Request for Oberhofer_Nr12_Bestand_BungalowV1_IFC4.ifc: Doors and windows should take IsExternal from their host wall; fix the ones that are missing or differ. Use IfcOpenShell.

First a look at what the model holds.

```python
import ifcopenshell
import ifcopenshell.util.element

model = ifcopenshell.open("Oberhofer_Nr12_Bestand_BungalowV1_IFC4.ifc")
print(model.schema)
seen = {}
for e in model.by_type("IfcDoor") + model.by_type("IfcWindow"):
    if not e.FillsVoids:
        continue
    host = e.FillsVoids[0].RelatingOpeningElement.VoidsElements[0].RelatingBuildingElement
    own = ifcopenshell.util.element.get_pset(e, f"Pset_{e.is_a()[3:].removesuffix('StandardCase')}Common", "IsExternal")
    wall = ifcopenshell.util.element.get_pset(host, "Pset_WallCommon", "IsExternal")
    seen[e.is_a(), own, wall] = seen.get((e.is_a(), own, wall), 0) + 1
for (cls, own, wall), count in sorted(seen.items(), key=str):
    print(count, cls, "IsExternal:", own, "| host wall:", wall)
```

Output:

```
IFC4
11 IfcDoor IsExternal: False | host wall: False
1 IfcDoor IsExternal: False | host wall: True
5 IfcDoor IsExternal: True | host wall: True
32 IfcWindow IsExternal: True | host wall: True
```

```python
import ifcopenshell
import ifcopenshell.api.pset
import ifcopenshell.util.element

model = ifcopenshell.open("Oberhofer_Nr12_Bestand_BungalowV1_IFC4.ifc")

count = 0
for ifc_class, pset_name in (("IfcDoor", "Pset_DoorCommon"), ("IfcWindow", "Pset_WindowCommon")):
    for e in model.by_type(ifc_class):
        if not e.FillsVoids:
            continue
        host = e.FillsVoids[0].RelatingOpeningElement.VoidsElements[0].RelatingBuildingElement
        external = ifcopenshell.util.element.get_pset(host, "Pset_WallCommon", "IsExternal")
        if external is None or ifcopenshell.util.element.get_pset(e, pset_name, "IsExternal") == external:
            continue
        pset = ifcopenshell.api.pset.add_pset(model, product=e, name=pset_name)
        ifcopenshell.api.pset.edit_pset(model, pset=pset, properties={"IsExternal": external})
        count += 1

print(count, "updated")

model.write("Oberhofer_Nr12_Bestand_BungalowV1_IFC4_v2.ifc")
```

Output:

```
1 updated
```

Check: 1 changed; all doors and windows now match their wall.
